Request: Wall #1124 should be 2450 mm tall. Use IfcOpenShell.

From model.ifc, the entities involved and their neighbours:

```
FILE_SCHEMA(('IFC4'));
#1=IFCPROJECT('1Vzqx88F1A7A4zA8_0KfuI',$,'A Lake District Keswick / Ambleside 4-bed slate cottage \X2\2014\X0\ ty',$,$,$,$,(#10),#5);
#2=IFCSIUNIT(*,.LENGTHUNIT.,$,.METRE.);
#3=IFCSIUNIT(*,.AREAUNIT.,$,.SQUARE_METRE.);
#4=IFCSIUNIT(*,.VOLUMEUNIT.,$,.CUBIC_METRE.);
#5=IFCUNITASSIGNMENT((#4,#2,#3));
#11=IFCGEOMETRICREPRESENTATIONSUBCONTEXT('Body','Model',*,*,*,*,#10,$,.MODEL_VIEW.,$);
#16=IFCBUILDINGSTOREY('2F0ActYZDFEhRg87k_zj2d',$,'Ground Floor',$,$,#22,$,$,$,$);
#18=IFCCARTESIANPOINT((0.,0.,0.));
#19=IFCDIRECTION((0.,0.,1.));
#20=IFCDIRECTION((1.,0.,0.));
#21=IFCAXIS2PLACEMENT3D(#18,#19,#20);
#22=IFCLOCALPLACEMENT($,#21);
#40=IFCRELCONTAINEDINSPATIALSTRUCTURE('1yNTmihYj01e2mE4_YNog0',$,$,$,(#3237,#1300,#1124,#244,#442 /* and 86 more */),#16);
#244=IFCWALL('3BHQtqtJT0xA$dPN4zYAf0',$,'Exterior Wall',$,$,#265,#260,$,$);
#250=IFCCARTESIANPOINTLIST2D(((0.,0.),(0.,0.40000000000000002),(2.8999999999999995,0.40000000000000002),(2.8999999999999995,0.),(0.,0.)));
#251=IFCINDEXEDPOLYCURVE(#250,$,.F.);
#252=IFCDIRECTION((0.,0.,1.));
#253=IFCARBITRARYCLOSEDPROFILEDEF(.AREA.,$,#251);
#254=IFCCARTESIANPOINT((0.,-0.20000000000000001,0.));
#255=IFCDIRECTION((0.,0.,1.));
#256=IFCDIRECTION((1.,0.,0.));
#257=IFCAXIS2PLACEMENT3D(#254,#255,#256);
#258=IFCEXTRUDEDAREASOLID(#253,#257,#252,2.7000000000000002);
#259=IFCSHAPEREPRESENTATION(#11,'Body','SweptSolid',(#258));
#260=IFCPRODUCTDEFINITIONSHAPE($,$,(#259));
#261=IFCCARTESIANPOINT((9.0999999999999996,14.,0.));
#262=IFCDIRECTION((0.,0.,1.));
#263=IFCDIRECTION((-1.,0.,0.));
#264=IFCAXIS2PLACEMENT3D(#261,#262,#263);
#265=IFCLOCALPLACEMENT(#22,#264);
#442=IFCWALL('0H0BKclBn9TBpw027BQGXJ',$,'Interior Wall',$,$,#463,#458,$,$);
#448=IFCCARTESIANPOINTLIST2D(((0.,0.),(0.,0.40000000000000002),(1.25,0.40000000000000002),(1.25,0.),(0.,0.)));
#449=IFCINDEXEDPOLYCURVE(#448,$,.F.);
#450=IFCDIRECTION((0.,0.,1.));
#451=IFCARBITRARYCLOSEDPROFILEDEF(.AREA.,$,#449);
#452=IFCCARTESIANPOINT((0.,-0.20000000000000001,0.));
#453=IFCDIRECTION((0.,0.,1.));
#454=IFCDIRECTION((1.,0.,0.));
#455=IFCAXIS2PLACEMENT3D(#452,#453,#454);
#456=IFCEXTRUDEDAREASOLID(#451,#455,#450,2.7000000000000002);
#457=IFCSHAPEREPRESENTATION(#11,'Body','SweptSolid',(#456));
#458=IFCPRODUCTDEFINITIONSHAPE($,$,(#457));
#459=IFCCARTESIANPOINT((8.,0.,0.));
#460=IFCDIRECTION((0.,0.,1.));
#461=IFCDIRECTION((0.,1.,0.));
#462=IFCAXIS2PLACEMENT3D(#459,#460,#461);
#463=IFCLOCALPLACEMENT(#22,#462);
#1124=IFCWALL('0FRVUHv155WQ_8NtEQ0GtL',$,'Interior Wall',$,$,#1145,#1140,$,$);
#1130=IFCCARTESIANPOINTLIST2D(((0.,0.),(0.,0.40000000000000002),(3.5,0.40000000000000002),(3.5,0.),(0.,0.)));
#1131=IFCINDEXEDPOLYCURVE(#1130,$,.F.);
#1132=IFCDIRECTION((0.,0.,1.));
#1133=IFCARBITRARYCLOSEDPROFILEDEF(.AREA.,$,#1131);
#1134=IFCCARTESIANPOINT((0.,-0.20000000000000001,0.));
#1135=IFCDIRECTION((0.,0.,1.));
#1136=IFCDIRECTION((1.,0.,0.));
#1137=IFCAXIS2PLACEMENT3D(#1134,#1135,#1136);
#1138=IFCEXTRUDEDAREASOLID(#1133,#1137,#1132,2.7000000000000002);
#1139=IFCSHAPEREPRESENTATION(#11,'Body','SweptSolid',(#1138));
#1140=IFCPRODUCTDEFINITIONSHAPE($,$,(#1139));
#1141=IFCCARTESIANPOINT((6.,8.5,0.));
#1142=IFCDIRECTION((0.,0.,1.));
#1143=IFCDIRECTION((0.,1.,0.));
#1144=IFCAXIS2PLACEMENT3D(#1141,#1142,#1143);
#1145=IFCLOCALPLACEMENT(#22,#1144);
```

```python
import ifcopenshell
import ifcopenshell.geom
import ifcopenshell.util.representation
import ifcopenshell.util.shape
import ifcopenshell.util.unit

model = ifcopenshell.open("model.ifc")
unit_scale = ifcopenshell.util.unit.calculate_unit_scale(model)
settings = ifcopenshell.geom.settings()


def volume(element):
    """Net volume in cubic metres, openings subtracted."""
    shape = ifcopenshell.geom.create_shape(settings, element)
    return ifcopenshell.util.shape.get_volume(shape.geometry)


wall = model.by_guid("0FRVUHv155WQ_8NtEQ0GtL")
before = volume(wall)

body = ifcopenshell.util.representation.get_representation(wall, "Model", "Body")
solid = body.Items[0]
old_height = solid.Depth
solid.Depth = 2.45 / unit_scale
after = volume(wall)

print(f"height {old_height:g} -> {solid.Depth:g}, volume {before:.3f} -> {after:.3f} m3")

model.write("model_updated.ifc")
```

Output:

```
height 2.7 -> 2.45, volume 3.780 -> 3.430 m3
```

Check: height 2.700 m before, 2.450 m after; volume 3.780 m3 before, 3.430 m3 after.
